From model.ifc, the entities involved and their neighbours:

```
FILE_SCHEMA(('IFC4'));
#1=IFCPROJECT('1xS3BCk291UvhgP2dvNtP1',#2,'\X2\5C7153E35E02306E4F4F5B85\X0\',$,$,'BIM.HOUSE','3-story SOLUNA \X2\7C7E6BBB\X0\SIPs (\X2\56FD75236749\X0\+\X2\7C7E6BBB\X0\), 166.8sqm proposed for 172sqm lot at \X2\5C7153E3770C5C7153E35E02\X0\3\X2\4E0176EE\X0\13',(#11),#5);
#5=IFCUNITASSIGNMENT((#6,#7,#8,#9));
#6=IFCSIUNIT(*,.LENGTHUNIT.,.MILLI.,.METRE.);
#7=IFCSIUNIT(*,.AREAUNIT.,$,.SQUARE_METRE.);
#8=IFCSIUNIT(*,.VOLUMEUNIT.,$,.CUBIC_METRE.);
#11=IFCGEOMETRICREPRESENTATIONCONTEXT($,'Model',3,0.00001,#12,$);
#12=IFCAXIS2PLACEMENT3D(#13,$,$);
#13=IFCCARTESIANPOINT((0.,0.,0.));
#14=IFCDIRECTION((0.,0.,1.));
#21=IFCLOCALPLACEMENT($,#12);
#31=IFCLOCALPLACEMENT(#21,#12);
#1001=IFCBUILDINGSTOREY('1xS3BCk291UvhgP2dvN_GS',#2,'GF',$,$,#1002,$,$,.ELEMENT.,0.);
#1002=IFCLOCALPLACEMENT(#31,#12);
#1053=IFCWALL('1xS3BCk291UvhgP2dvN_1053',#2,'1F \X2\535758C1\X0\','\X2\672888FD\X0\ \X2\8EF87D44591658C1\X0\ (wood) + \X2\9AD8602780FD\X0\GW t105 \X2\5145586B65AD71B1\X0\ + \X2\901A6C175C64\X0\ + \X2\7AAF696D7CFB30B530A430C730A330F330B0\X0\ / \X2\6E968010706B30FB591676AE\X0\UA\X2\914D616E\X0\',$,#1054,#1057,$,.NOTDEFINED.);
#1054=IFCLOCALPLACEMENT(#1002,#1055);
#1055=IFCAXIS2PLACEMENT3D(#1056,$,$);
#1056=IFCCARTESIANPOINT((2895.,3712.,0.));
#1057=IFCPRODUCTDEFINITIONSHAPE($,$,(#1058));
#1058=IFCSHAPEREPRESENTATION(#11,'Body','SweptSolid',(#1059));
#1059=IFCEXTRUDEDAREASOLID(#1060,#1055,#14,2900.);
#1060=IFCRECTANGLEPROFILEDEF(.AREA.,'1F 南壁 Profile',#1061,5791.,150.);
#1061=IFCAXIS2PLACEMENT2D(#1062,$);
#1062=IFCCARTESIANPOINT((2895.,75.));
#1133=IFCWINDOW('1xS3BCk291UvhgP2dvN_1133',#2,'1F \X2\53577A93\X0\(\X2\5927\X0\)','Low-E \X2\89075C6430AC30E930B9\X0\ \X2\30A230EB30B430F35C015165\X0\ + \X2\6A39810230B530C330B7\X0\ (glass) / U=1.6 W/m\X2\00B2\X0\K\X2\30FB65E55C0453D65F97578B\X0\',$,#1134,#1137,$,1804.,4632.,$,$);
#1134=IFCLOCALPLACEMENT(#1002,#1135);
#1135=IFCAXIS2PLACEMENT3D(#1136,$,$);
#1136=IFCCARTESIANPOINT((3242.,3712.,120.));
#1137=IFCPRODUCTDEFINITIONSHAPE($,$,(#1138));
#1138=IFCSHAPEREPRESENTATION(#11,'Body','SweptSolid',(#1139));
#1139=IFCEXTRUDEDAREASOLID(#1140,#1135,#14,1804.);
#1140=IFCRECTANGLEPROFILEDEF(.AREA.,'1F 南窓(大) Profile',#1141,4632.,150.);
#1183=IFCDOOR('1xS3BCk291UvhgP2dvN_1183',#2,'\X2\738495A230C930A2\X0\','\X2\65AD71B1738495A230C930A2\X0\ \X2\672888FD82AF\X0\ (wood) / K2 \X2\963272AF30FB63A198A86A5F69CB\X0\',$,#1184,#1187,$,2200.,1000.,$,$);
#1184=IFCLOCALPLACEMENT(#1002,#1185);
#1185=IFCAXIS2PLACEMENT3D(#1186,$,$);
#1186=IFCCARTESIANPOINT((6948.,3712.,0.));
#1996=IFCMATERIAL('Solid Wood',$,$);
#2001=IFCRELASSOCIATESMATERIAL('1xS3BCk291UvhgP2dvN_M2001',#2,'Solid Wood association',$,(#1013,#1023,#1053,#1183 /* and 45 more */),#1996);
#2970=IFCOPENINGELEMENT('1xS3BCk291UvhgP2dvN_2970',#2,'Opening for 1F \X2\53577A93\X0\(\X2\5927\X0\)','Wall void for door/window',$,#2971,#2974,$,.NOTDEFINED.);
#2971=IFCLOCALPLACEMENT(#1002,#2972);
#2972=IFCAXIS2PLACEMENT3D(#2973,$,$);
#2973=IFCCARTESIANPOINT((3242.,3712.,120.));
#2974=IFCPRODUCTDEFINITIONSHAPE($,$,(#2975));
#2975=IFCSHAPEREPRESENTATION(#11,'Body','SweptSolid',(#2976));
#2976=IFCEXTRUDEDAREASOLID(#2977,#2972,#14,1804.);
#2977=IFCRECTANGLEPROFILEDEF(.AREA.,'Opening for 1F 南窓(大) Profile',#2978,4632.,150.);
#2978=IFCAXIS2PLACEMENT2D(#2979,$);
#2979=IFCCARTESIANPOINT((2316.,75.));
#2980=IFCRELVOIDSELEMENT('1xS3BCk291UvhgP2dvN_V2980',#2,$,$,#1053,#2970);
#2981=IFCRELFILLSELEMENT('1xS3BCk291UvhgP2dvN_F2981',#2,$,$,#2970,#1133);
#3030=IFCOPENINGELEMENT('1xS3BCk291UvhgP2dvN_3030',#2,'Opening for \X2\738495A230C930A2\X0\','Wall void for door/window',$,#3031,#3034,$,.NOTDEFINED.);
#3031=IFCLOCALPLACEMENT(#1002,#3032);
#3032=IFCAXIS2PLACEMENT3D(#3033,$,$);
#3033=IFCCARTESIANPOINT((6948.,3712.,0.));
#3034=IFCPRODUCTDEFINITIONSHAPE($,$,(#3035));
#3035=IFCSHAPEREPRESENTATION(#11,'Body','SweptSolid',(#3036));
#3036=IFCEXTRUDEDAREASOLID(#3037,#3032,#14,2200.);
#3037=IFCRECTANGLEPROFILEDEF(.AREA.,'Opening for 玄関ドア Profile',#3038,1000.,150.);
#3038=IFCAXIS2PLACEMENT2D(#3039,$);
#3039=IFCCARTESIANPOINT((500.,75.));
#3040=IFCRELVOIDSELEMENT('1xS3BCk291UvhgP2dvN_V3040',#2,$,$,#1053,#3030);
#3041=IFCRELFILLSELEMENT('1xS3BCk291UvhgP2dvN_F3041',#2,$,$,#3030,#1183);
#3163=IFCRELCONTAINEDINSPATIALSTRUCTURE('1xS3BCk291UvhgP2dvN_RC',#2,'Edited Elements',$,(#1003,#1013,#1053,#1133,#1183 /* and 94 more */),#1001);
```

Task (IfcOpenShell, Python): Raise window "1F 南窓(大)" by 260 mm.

```python
import numpy as np
import ifcopenshell
import ifcopenshell.api.geometry
import ifcopenshell.util.placement
import ifcopenshell.util.unit

model = ifcopenshell.open("model.ifc")
unit_scale = ifcopenshell.util.unit.calculate_unit_scale(model)

window = model.by_guid("1xS3BCk291UvhgP2dvN_1133")
opening = window.FillsVoids[0].RelatingOpeningElement
dz = 0.26 / unit_scale

shift = np.array([0.0, 0.0, dz])
# The window is not placed relative to its opening, so move both.
for product in (opening, window):
    matrix = ifcopenshell.util.placement.get_local_placement(product.ObjectPlacement)
    matrix[:3, 3] += shift
    ifcopenshell.api.geometry.edit_object_placement(model, product=product, matrix=matrix, is_si=False)

print(f"moved by {dz * unit_scale:+.3f} m")

model.write("model-out.ifc")
```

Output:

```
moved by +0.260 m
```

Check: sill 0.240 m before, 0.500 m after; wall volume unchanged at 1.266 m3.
